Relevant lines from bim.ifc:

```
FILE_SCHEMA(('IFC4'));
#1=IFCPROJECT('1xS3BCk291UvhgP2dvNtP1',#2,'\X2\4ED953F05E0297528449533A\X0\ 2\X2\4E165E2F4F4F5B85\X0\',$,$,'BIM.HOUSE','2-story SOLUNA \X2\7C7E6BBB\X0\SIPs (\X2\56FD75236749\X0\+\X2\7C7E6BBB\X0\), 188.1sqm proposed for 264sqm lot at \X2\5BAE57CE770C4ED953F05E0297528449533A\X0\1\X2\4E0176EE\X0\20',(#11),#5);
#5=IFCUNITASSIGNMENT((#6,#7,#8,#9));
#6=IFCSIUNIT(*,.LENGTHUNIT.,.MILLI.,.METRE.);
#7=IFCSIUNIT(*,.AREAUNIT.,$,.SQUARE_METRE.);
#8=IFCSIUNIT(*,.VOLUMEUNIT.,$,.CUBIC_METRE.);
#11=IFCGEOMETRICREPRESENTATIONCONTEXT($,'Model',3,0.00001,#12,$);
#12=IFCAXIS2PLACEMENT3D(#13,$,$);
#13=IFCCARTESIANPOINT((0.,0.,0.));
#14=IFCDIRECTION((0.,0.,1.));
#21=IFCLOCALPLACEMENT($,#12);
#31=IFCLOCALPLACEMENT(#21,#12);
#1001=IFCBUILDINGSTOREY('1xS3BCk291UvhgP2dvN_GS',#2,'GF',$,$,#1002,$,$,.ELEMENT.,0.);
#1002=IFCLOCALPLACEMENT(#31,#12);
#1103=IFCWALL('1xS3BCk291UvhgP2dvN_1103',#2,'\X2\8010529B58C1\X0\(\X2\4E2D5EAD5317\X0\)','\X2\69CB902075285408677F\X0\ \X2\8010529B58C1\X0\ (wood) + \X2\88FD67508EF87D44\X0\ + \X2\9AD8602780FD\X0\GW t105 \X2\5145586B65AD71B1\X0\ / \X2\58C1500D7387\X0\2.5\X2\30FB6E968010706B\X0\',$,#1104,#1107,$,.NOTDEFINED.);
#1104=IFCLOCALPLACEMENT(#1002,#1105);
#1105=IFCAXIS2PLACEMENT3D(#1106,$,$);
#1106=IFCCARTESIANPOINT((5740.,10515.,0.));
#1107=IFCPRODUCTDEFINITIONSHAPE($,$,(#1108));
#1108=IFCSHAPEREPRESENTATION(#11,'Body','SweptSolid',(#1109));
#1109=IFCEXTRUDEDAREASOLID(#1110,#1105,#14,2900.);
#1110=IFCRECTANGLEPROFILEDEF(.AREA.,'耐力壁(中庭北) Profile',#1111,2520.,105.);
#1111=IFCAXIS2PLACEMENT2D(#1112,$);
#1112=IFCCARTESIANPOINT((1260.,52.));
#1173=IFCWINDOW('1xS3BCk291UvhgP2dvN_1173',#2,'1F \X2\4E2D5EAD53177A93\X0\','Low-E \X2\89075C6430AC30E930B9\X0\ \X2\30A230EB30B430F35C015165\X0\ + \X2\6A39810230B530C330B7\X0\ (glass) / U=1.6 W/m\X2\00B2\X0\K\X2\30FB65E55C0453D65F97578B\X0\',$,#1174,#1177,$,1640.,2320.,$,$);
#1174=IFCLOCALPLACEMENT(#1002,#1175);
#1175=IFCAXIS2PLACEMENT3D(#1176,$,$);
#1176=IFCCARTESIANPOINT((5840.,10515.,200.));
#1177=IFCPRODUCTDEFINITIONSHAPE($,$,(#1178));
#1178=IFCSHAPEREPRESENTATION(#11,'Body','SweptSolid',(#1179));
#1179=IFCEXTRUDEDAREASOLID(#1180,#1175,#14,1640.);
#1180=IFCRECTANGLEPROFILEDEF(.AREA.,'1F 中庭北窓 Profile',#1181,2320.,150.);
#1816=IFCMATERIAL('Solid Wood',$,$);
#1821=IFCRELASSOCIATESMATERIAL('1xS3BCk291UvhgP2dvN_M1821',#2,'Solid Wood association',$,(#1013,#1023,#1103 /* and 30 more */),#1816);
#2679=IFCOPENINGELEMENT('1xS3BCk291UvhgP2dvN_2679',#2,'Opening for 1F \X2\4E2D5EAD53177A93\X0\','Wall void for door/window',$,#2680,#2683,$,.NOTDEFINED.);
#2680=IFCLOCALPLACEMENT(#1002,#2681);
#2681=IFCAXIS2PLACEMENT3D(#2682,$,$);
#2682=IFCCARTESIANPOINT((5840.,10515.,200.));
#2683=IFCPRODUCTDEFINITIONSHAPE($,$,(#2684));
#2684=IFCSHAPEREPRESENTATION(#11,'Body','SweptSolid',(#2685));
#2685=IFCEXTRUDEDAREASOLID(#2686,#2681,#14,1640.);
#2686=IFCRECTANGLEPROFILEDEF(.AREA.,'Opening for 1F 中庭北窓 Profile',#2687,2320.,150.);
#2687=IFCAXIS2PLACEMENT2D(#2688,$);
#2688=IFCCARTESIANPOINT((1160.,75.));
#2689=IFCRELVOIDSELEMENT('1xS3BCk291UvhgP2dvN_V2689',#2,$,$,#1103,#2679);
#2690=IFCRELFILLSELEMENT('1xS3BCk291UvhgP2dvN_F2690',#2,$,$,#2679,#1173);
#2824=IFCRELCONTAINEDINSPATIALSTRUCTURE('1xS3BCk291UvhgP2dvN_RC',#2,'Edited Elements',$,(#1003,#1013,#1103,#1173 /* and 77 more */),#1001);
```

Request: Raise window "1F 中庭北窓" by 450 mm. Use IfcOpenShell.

```python
import numpy as np
import ifcopenshell
import ifcopenshell.api.geometry
import ifcopenshell.util.placement
import ifcopenshell.util.unit

model = ifcopenshell.open("bim.ifc")
unit_scale = ifcopenshell.util.unit.calculate_unit_scale(model)

window = model.by_guid("1xS3BCk291UvhgP2dvN_1173")
opening = window.FillsVoids[0].RelatingOpeningElement
dz = 0.45 / unit_scale

shift = np.array([0.0, 0.0, dz])
# The window is not placed relative to its opening, so move both.
for product in (opening, window):
    matrix = ifcopenshell.util.placement.get_local_placement(product.ObjectPlacement)
    matrix[:3, 3] += shift
    ifcopenshell.api.geometry.edit_object_placement(model, product=product, matrix=matrix, is_si=False)

print(f"moved by {dz * unit_scale:+.3f} m")

model.write("bim_v2.ifc")
```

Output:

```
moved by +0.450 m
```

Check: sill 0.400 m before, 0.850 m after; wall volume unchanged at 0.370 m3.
